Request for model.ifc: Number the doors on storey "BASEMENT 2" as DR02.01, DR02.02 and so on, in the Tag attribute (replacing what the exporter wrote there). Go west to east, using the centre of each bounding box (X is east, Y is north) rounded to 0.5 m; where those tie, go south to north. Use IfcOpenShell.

First a look at what the model holds.

```python
import ifcopenshell
import ifcopenshell.util.element
import ifcopenshell.util.placement

model = ifcopenshell.open("model.ifc")
print(model.schema)
storey = next(s for s in model.by_type("IfcBuildingStorey") if s.Name == "BASEMENT 2")
doors = [e for e in ifcopenshell.util.element.get_decomposition(storey) if e.is_a("IfcDoor")]
for e in sorted(doors, key=lambda e: e.id()):
    origin = ifcopenshell.util.placement.get_local_placement(e.ObjectPlacement)[:3, 3]
    print(e.id(), e.Tag, e.Name, origin.round(2) + 0.0, sep=" | ")
```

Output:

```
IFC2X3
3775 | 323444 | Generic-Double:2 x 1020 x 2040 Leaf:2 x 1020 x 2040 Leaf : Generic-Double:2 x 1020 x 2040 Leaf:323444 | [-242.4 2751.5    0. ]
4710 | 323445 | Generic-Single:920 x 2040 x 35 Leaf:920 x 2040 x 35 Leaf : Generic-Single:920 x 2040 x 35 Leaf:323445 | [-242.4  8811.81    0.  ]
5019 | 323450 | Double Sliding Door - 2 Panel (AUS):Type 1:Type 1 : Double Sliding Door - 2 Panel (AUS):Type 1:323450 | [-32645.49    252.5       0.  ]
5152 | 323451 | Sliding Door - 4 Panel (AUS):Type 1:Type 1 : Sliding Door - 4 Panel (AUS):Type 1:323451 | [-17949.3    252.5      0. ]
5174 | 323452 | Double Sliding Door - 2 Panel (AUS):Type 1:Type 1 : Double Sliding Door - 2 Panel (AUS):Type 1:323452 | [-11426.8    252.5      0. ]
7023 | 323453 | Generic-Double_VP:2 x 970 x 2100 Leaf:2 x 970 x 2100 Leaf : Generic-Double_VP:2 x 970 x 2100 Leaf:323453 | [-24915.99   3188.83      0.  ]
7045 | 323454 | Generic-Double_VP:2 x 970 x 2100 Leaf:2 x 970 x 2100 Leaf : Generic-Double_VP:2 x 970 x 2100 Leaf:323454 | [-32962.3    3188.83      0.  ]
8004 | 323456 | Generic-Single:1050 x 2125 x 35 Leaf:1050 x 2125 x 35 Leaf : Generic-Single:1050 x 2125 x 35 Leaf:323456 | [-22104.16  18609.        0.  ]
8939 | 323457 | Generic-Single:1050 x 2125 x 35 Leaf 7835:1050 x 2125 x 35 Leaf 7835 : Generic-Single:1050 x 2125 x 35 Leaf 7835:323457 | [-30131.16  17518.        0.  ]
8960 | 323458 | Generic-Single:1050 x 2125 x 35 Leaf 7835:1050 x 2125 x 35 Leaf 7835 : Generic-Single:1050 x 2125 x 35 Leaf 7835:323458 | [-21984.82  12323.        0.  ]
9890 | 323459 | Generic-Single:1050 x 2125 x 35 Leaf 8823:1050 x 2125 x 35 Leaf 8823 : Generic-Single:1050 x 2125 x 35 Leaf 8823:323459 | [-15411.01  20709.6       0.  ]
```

```python
import ifcopenshell
import ifcopenshell.geom
import ifcopenshell.util.element
import ifcopenshell.util.shape

model = ifcopenshell.open("model.ifc")
settings = ifcopenshell.geom.settings()
settings.set("use-world-coords", True)


def centre(element):
    shape = ifcopenshell.geom.create_shape(settings, element)
    return ifcopenshell.util.shape.get_bbox_centroid(shape.geometry)


storey = next(s for s in model.by_type("IfcBuildingStorey") if s.Name == "BASEMENT 2")
doors = [e for e in ifcopenshell.util.element.get_decomposition(storey) if e.is_a("IfcDoor")]

# Insertion points can sit at a corner or the storey origin, so sort by the geometry (in metres).
centres = {e: centre(e) for e in doors}
doors.sort(key=lambda e: (round(centres[e][0] / 0.5), centres[e][1]))

for i, e in enumerate(doors, start=1):
    number = f"DR02.{i:02d}"
    e.Tag = number
    print(e.id(), number)

model.write("model_rev.ifc")
```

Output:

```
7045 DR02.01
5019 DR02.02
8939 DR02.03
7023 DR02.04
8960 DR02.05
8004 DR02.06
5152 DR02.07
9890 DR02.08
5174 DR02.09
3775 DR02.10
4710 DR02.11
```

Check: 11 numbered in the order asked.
